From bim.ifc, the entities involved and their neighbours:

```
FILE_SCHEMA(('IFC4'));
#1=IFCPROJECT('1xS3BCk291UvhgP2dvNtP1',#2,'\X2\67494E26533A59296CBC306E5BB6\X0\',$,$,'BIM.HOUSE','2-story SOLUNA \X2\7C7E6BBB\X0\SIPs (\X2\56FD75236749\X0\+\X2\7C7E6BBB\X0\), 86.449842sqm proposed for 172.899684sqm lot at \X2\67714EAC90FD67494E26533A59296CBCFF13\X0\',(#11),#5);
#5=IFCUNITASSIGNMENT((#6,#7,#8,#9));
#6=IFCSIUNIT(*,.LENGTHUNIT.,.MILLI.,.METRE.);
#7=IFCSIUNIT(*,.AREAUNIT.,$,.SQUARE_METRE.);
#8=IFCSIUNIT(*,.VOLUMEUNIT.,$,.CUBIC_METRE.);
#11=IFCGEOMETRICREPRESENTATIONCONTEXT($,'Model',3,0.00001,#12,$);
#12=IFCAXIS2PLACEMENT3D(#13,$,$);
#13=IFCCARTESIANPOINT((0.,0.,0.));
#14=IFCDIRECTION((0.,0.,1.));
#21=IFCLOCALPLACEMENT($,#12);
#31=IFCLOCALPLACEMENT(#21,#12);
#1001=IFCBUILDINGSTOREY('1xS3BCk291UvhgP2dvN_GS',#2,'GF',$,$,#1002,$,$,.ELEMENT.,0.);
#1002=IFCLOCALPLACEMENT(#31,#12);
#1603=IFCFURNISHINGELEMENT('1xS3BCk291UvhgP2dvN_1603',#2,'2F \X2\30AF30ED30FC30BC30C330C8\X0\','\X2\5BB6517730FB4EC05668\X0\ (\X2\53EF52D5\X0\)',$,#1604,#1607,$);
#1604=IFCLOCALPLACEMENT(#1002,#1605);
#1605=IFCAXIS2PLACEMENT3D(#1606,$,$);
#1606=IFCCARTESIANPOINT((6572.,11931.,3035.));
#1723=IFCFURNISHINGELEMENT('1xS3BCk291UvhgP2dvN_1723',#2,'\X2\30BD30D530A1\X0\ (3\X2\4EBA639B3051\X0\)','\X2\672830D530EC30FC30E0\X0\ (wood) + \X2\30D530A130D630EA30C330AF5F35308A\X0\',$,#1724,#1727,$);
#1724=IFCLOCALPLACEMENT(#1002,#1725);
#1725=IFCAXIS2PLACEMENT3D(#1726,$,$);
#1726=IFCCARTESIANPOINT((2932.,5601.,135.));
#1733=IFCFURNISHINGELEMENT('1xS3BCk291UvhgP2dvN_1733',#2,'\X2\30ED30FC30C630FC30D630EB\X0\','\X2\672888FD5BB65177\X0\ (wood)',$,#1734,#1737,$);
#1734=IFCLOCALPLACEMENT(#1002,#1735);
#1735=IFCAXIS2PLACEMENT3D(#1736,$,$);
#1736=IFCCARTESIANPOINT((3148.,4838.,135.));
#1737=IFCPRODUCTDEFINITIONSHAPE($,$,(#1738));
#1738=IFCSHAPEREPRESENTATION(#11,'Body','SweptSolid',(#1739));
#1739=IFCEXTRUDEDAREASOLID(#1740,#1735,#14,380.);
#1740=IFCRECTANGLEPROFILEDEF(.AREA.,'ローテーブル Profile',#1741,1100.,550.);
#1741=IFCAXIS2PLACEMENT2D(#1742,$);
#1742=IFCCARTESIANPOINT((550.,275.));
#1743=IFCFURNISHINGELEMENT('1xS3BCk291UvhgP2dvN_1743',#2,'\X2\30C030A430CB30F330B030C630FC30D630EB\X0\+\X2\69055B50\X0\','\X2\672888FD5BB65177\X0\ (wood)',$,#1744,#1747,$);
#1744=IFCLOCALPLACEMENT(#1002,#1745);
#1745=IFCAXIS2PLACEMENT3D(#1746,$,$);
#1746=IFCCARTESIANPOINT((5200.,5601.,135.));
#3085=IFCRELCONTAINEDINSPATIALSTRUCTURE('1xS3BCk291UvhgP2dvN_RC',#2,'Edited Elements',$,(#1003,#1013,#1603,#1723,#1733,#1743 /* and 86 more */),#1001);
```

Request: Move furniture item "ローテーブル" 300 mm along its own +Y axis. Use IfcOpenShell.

```python
import ifcopenshell
import ifcopenshell.api.geometry
import ifcopenshell.util.placement

model = ifcopenshell.open("bim.ifc")

item = model.by_id(1733)
matrix = ifcopenshell.util.placement.get_local_placement(item.ObjectPlacement)
matrix[:3, 3] += matrix[:3, 1] * 300.0
ifcopenshell.api.geometry.edit_object_placement(model, product=item, matrix=matrix, is_si=False)

print(ifcopenshell.util.placement.get_local_placement(item.ObjectPlacement).round(3) + 0.0)

model.write("bim_updated.ifc")
```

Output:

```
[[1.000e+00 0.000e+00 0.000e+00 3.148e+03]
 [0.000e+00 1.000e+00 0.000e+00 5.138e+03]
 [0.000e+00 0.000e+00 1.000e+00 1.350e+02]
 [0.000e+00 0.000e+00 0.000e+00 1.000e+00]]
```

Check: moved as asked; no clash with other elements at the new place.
